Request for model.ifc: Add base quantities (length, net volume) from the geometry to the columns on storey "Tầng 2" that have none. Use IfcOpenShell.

First a look at what the model holds.

```python
import ifcopenshell
import ifcopenshell.util.element
import ifcopenshell.util.unit

model = ifcopenshell.open("model.ifc")
print(model.schema)
for unit_type in ("LENGTHUNIT", "AREAUNIT", "VOLUMEUNIT"):
    print(unit_type, ifcopenshell.util.unit.calculate_unit_scale(model, unit_type))
storey = next(s for s in model.by_type("IfcBuildingStorey") if s.Name == "Tầng 2")
columns = [e for e in ifcopenshell.util.element.get_decomposition(storey) if e.is_a("IfcColumn")]
for e in sorted(columns, key=lambda e: e.id()):
    print(e.id(), e.is_a(), e.Name, list(ifcopenshell.util.element.get_psets(e, qtos_only=True)), sep=" | ")
```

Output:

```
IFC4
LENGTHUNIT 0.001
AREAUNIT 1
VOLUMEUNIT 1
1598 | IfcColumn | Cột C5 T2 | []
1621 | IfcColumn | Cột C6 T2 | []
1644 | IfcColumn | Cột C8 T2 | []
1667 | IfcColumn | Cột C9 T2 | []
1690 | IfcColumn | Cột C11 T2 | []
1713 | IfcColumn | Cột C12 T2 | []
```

```python
import ifcopenshell
import ifcopenshell.api.pset
import ifcopenshell.geom
import ifcopenshell.util.element
import ifcopenshell.util.shape
import ifcopenshell.util.unit

model = ifcopenshell.open("model.ifc")
unit_scale = ifcopenshell.util.unit.calculate_unit_scale(model)
volume_scale = ifcopenshell.util.unit.calculate_unit_scale(model, "VOLUMEUNIT")
settings = ifcopenshell.geom.settings()

storey = next(s for s in model.by_type("IfcBuildingStorey") if s.Name == "Tầng 2")
columns = [e for e in ifcopenshell.util.element.get_decomposition(storey) if e.is_a("IfcColumn")]

for e in sorted(columns, key=lambda e: e.id()):
    if ifcopenshell.util.element.get_psets(e, qtos_only=True, should_inherit=False):
        continue
    # Geometry comes back in metres, in the element's own axes.
    shape = ifcopenshell.geom.create_shape(settings, e)
    values = {
        "Length": ifcopenshell.util.shape.get_z(shape.geometry) / unit_scale,
        "NetVolume": ifcopenshell.util.shape.get_volume(shape.geometry) / volume_scale,
    }
    qto = ifcopenshell.api.pset.add_qto(model, product=e, name="Qto_ColumnBaseQuantities")
    ifcopenshell.api.pset.edit_qto(model, qto=qto, properties=values)
    print(e.id(), {k: round(v, 3) for k, v in values.items()})

model.write("model-out.ifc")
```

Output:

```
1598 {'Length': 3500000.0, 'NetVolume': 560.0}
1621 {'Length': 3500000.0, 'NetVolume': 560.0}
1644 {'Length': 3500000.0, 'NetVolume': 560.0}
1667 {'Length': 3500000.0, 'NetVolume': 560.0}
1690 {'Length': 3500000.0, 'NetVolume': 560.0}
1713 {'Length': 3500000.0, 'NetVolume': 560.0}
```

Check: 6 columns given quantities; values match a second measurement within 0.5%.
